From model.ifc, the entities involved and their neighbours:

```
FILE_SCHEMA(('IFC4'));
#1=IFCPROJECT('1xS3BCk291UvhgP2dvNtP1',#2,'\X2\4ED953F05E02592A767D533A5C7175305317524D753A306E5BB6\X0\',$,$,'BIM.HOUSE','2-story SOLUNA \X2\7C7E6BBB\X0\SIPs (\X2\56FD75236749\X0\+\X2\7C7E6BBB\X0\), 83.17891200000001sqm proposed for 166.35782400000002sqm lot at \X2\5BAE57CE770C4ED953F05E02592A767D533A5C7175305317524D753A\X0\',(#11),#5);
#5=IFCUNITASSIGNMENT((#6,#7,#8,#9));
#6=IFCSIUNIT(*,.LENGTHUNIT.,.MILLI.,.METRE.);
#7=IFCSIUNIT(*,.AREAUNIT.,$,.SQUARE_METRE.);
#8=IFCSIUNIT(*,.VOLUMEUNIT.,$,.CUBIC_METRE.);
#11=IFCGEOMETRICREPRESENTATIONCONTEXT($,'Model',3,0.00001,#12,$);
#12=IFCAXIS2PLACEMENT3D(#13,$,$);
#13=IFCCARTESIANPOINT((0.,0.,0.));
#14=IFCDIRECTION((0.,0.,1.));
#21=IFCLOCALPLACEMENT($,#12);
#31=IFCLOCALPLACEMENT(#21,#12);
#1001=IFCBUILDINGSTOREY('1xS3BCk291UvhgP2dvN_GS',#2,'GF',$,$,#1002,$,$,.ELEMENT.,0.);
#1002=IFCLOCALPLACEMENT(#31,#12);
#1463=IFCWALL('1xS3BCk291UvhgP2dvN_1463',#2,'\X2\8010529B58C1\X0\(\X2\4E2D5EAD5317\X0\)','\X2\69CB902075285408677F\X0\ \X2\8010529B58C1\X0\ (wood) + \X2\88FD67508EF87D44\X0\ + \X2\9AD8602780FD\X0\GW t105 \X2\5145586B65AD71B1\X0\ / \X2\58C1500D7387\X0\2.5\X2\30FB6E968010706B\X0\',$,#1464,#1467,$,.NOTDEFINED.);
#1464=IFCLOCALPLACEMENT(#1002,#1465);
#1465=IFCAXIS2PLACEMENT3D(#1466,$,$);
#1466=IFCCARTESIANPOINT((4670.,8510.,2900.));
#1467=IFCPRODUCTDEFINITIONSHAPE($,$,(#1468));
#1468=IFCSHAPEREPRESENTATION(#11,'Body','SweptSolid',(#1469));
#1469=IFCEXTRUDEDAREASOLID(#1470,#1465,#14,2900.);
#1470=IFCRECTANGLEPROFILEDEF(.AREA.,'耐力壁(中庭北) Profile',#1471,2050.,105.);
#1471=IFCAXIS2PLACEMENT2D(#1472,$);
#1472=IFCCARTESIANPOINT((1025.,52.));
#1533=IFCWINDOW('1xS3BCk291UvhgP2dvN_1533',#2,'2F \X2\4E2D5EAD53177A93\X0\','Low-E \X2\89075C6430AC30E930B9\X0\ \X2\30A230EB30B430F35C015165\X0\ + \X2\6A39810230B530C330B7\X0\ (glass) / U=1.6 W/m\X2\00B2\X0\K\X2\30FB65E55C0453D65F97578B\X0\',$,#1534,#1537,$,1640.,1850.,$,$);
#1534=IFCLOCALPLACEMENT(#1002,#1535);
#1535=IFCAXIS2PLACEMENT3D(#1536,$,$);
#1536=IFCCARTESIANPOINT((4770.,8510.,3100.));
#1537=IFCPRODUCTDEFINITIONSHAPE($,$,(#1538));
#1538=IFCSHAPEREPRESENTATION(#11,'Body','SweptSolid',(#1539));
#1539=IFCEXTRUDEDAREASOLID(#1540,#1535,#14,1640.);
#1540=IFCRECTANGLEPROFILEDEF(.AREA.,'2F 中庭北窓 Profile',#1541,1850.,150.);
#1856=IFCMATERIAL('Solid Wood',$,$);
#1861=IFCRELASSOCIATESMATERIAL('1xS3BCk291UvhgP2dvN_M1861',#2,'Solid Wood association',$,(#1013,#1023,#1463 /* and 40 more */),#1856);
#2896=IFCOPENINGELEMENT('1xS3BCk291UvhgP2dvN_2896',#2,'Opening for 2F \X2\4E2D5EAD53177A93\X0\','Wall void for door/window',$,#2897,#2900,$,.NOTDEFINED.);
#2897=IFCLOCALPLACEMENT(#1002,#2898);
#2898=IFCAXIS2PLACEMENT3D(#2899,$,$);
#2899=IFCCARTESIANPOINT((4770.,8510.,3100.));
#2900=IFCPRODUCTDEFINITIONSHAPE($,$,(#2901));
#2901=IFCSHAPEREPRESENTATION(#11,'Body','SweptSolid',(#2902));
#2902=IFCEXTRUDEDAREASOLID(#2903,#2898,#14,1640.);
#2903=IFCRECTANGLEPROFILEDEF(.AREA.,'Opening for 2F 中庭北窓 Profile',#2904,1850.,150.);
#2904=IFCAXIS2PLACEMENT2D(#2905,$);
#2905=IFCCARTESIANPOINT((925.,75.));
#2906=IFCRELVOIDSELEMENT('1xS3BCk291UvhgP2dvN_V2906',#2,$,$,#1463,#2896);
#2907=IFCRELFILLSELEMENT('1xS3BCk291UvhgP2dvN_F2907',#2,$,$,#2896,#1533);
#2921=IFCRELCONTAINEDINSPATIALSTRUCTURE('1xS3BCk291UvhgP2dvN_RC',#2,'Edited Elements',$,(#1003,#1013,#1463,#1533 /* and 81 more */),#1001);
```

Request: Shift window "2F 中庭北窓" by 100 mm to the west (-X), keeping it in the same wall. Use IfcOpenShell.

```python
import ifcopenshell
import ifcopenshell.api.geometry
import ifcopenshell.util.placement
import ifcopenshell.util.unit

model = ifcopenshell.open("model.ifc")
unit_scale = ifcopenshell.util.unit.calculate_unit_scale(model)

window = model.by_guid("1xS3BCk291UvhgP2dvN_1533")
opening = window.FillsVoids[0].RelatingOpeningElement
wall = opening.VoidsElements[0].RelatingBuildingElement

wall_matrix = ifcopenshell.util.placement.get_local_placement(wall.ObjectPlacement)
shift = wall_matrix[:3, 0] * -0.1 / unit_scale
before = ifcopenshell.util.placement.get_local_placement(window.ObjectPlacement)[:3, 3].copy()

# The window is not placed relative to its opening, so move both.
for product in (opening, window):
    matrix = ifcopenshell.util.placement.get_local_placement(product.ObjectPlacement)
    matrix[:3, 3] += shift
    ifcopenshell.api.geometry.edit_object_placement(model, product=product, matrix=matrix, is_si=False)

after = ifcopenshell.util.placement.get_local_placement(window.ObjectPlacement)[:3, 3]
print("window moved by", (after - before).round(3) + 0.0)

model.write("model_rev.ifc")
```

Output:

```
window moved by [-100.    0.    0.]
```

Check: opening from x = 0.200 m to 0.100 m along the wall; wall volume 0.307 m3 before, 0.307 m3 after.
